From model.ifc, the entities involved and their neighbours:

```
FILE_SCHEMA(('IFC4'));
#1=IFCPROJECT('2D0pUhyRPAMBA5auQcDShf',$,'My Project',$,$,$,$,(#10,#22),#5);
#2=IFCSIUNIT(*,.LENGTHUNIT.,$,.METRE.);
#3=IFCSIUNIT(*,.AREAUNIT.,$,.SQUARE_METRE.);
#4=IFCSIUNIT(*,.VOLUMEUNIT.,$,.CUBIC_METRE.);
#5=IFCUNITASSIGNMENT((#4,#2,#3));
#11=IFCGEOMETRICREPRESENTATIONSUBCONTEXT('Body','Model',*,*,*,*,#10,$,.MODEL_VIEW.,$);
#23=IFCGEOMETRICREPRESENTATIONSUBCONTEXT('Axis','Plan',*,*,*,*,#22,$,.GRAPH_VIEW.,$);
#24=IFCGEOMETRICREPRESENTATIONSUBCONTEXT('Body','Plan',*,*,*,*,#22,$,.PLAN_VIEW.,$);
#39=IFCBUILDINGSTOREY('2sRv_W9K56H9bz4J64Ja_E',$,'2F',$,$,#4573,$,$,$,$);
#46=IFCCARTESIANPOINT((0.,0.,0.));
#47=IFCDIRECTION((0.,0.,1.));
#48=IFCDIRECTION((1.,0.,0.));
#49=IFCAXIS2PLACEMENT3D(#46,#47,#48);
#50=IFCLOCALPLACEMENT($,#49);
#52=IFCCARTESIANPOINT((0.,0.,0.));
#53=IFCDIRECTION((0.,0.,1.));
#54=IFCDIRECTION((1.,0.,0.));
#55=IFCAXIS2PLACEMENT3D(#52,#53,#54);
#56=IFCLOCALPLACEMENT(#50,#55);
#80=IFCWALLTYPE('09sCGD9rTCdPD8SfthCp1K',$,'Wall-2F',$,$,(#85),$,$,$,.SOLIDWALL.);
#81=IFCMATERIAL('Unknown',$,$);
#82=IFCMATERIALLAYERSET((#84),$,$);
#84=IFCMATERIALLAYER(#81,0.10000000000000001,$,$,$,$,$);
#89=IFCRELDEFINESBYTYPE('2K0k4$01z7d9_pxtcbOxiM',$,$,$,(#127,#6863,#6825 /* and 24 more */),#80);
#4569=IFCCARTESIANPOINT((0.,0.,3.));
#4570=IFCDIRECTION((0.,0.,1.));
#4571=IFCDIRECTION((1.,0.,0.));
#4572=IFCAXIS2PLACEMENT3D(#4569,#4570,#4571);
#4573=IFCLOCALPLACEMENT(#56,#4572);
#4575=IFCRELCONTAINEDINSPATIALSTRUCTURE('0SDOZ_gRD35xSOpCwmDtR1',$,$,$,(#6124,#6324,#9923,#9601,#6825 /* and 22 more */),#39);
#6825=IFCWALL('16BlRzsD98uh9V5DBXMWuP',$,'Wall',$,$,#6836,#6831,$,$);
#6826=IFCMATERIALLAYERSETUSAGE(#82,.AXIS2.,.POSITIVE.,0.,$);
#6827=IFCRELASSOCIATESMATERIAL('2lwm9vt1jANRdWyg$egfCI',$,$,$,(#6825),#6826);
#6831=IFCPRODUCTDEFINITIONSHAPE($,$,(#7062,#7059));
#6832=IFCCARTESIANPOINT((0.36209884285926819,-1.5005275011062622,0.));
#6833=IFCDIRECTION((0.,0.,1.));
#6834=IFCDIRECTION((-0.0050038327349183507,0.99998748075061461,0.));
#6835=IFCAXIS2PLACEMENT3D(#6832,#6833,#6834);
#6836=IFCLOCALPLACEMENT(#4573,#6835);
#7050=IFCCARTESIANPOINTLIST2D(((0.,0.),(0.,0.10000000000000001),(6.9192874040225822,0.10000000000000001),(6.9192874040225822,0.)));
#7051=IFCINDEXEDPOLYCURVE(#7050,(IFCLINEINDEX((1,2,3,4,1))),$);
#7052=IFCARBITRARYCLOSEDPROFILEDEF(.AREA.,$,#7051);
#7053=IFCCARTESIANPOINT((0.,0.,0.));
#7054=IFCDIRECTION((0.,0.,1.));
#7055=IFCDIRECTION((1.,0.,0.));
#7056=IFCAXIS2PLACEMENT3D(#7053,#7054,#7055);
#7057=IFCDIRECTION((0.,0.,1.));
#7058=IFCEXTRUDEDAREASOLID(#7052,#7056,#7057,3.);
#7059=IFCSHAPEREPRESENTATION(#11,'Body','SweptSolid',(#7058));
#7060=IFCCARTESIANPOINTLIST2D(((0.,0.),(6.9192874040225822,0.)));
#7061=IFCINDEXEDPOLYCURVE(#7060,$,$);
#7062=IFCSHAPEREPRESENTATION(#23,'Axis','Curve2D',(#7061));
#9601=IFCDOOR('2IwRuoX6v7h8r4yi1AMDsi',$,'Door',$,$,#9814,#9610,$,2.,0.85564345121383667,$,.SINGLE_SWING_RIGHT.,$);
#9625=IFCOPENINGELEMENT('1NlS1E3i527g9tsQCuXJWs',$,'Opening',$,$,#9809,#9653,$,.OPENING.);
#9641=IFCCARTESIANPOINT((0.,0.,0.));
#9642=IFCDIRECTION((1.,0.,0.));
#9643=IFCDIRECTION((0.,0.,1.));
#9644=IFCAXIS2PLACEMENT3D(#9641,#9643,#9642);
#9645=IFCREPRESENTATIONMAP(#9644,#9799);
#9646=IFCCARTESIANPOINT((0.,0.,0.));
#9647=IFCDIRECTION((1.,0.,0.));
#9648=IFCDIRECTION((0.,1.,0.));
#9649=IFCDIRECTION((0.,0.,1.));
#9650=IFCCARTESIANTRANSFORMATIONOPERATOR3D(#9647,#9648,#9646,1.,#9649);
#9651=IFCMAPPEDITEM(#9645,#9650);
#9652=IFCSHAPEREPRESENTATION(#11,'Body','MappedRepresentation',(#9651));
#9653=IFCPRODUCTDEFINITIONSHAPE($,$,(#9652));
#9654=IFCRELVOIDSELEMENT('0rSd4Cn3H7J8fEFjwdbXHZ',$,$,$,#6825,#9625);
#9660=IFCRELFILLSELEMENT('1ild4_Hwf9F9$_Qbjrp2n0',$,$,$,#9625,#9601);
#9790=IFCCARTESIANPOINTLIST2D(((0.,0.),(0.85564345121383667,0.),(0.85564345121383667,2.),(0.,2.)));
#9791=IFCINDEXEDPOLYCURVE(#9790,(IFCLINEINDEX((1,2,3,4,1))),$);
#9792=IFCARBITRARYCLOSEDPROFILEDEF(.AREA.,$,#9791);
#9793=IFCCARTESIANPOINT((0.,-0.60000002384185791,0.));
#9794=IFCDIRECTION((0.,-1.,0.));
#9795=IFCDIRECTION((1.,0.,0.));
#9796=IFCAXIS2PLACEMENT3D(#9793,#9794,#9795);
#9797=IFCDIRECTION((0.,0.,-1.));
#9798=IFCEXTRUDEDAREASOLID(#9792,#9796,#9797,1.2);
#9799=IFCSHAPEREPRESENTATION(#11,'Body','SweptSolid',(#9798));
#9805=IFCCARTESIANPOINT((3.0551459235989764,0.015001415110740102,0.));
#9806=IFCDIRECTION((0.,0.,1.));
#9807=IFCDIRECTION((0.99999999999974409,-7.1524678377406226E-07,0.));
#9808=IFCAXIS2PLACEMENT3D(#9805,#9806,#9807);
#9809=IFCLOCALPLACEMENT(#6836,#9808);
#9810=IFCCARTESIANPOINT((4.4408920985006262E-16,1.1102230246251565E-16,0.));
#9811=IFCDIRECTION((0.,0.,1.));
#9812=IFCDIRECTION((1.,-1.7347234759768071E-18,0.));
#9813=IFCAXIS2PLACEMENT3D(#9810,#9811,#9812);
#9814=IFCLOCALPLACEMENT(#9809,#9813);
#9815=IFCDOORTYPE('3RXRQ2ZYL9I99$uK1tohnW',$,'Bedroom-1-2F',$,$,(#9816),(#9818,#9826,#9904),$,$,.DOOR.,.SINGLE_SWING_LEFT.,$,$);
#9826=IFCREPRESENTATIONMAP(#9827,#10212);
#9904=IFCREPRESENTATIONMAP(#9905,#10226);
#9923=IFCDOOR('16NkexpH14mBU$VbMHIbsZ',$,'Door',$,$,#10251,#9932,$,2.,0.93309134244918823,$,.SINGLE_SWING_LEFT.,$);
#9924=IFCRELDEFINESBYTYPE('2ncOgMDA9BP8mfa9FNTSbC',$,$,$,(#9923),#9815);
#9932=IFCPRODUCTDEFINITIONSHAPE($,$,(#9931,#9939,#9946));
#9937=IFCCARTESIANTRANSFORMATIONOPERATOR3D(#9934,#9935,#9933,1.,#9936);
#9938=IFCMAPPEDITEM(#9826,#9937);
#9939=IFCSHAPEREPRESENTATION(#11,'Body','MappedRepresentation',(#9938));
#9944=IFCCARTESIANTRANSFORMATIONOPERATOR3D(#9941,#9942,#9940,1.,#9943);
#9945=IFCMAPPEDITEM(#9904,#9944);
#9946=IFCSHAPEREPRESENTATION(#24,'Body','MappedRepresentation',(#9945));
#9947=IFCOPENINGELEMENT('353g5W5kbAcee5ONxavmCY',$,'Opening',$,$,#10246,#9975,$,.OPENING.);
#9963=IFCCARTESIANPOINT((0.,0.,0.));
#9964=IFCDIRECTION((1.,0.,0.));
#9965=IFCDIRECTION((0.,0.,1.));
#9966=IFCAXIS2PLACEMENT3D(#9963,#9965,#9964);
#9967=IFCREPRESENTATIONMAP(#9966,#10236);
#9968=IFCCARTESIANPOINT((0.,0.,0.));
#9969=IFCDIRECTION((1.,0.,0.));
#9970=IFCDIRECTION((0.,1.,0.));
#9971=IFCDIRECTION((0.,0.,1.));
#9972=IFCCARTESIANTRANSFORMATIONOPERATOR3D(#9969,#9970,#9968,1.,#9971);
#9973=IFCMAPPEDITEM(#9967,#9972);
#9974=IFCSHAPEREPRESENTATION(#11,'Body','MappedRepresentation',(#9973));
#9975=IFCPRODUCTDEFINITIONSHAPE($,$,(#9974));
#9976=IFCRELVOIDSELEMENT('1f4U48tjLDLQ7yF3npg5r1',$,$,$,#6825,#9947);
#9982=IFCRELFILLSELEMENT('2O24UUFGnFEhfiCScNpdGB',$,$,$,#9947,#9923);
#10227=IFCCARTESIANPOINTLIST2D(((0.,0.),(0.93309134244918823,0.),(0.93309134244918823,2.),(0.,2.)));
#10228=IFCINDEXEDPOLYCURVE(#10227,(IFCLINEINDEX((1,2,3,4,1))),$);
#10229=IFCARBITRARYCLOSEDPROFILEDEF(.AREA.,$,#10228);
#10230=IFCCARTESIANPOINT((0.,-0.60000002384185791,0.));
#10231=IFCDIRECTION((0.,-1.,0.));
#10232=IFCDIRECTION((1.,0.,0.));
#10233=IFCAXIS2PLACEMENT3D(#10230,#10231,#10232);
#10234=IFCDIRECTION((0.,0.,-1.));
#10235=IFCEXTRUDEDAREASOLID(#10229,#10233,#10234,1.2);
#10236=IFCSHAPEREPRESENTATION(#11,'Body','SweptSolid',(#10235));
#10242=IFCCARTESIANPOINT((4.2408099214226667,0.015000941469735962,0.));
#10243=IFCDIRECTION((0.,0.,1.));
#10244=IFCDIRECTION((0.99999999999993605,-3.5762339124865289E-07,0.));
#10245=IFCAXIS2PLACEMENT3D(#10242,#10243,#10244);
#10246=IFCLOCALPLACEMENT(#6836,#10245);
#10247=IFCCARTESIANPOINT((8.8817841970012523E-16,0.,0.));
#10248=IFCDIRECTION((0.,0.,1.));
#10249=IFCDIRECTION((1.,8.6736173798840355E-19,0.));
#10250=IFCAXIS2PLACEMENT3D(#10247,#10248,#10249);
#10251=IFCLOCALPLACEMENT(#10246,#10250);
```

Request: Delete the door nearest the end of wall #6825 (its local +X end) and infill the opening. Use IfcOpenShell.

```python
import ifcopenshell
import ifcopenshell.api.feature
import ifcopenshell.api.root
import ifcopenshell.geom
import ifcopenshell.util.shape

model = ifcopenshell.open("model.ifc")
settings = ifcopenshell.geom.settings()


def volume(element):
    """Net volume in cubic metres, openings subtracted."""
    shape = ifcopenshell.geom.create_shape(settings, element)
    return ifcopenshell.util.shape.get_volume(shape.geometry)


door = model.by_id(9923)
opening = door.FillsVoids[0].RelatingOpeningElement
wall = opening.VoidsElements[0].RelatingBuildingElement
before = volume(wall)

ifcopenshell.api.root.remove_product(model, product=door)
ifcopenshell.api.feature.remove_feature(model, feature=opening)

after = volume(wall)

print(f"wall volume {before:.3f} -> {after:.3f} m3")

model.write("model-out.ifc")
```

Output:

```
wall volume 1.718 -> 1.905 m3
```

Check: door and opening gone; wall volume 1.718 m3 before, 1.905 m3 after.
